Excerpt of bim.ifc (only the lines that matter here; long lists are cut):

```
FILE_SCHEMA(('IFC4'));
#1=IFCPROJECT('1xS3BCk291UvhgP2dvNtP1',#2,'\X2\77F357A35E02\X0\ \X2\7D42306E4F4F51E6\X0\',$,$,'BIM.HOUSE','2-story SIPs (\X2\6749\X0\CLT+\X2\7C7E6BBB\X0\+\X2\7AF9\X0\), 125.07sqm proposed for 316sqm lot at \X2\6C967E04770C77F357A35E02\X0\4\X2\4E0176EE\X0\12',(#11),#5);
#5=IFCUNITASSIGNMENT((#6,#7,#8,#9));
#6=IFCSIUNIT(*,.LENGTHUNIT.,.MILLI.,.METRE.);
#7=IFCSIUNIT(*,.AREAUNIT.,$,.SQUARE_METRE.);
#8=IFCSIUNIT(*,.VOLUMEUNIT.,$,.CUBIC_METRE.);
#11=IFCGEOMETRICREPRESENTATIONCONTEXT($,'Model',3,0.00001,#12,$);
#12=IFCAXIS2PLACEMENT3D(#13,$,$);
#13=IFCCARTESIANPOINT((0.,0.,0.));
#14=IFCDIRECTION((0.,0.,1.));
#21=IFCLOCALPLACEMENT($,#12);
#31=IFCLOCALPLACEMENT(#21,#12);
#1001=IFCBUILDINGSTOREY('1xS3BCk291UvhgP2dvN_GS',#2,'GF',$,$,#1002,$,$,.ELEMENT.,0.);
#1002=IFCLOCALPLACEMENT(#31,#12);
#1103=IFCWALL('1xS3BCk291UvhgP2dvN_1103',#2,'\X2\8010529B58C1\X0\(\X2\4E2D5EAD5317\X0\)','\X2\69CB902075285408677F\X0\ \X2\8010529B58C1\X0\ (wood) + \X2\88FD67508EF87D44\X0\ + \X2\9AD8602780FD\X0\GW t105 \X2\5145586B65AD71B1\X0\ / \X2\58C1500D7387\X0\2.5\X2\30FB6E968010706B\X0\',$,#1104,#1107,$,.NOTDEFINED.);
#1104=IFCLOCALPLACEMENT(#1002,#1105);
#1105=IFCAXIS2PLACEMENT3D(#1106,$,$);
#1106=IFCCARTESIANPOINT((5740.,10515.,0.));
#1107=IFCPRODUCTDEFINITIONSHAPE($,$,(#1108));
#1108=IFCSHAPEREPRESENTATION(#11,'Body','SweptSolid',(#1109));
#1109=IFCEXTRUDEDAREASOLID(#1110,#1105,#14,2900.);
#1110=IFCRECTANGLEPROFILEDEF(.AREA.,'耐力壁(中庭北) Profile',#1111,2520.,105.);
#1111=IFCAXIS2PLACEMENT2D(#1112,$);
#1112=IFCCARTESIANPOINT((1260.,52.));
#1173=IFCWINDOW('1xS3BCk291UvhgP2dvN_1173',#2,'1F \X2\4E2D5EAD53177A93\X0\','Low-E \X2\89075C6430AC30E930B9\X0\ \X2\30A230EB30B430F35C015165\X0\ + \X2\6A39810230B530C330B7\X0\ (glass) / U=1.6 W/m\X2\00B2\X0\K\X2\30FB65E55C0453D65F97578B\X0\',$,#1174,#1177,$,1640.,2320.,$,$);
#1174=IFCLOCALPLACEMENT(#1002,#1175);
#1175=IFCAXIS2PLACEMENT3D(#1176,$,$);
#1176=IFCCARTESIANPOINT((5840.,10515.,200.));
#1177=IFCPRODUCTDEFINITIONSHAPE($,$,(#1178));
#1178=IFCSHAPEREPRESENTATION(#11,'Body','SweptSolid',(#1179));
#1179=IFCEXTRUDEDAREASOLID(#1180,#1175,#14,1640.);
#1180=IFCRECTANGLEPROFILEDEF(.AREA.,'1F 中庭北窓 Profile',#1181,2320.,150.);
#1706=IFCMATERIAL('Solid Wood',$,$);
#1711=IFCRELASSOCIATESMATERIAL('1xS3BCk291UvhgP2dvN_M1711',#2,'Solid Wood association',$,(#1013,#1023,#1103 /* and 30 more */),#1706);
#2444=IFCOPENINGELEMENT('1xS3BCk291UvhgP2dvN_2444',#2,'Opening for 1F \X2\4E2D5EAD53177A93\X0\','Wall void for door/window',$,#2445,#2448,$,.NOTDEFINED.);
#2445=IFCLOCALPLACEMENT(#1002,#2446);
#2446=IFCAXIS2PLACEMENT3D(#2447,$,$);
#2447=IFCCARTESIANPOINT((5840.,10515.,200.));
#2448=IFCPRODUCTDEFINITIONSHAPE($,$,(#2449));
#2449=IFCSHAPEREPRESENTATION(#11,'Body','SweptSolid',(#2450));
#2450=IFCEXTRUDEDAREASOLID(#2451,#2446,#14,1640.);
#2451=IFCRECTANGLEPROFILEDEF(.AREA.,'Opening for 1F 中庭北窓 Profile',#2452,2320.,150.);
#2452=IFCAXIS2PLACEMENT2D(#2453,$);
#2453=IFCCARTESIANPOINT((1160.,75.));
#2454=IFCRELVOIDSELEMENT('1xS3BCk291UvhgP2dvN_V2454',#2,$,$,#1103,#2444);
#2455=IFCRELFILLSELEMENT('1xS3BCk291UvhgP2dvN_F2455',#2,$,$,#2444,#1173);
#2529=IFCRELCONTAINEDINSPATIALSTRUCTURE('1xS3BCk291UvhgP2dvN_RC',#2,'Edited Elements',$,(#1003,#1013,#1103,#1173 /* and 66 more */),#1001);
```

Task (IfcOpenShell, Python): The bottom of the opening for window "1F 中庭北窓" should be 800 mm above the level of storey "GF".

```python
import numpy as np
import ifcopenshell
import ifcopenshell.api.geometry
import ifcopenshell.geom
import ifcopenshell.util.element
import ifcopenshell.util.placement
import ifcopenshell.util.shape
import ifcopenshell.util.unit

model = ifcopenshell.open("bim.ifc")
unit_scale = ifcopenshell.util.unit.calculate_unit_scale(model)

window = model.by_guid("1xS3BCk291UvhgP2dvN_1173")
opening = window.FillsVoids[0].RelatingOpeningElement
storey = ifcopenshell.util.element.get_container(window, ifc_class="IfcBuildingStorey")
level = ifcopenshell.util.placement.get_local_placement(storey.ObjectPlacement)[2, 3]

# The opening's origin need not be at the sill, so measure its lowest point.
shape = ifcopenshell.geom.create_shape(ifcopenshell.geom.settings(), opening)
bottom = ifcopenshell.util.shape.get_shape_bottom_elevation(shape, shape.geometry) / unit_scale
dz = level + 0.8 / unit_scale - bottom

shift = np.array([0.0, 0.0, dz])
# The window is not placed relative to its opening, so move both.
for product in (opening, window):
    matrix = ifcopenshell.util.placement.get_local_placement(product.ObjectPlacement)
    matrix[:3, 3] += shift
    ifcopenshell.api.geometry.edit_object_placement(model, product=product, matrix=matrix, is_si=False)

print(f"moved by {dz * unit_scale:+.3f} m")

model.write("bim_rev.ifc")
```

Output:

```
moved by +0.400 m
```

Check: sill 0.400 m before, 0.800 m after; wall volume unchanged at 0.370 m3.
